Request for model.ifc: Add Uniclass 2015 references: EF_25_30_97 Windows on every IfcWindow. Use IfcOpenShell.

First a look at what the model holds.

```python
import ifcopenshell

model = ifcopenshell.open("model.ifc")
print(model.schema)
print("classifications:", [c.Name for c in model.by_type("IfcClassification")])
for ifc_class in ("IfcDoor", "IfcRoof", "IfcStair", "IfcWall", "IfcWindow"):
    print(ifc_class, len(model.by_type(ifc_class)))
```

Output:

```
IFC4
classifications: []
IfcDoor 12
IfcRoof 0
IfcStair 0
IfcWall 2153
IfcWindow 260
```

```python
import ifcopenshell
import ifcopenshell.api.classification

model = ifcopenshell.open("model.ifc")

system = ifcopenshell.api.classification.add_classification(model, classification="Uniclass 2015")

codes = {
    "IfcWindow": ("EF_25_30_97", "Windows"),
}
for ifc_class, (code, name) in codes.items():
    products = model.by_type(ifc_class)
    ifcopenshell.api.classification.add_reference(
        model, products=products, classification=system, identification=code, name=name
    )
    print(code, len(products))

model.write("model-out.ifc")
```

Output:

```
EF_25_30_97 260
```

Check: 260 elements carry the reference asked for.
